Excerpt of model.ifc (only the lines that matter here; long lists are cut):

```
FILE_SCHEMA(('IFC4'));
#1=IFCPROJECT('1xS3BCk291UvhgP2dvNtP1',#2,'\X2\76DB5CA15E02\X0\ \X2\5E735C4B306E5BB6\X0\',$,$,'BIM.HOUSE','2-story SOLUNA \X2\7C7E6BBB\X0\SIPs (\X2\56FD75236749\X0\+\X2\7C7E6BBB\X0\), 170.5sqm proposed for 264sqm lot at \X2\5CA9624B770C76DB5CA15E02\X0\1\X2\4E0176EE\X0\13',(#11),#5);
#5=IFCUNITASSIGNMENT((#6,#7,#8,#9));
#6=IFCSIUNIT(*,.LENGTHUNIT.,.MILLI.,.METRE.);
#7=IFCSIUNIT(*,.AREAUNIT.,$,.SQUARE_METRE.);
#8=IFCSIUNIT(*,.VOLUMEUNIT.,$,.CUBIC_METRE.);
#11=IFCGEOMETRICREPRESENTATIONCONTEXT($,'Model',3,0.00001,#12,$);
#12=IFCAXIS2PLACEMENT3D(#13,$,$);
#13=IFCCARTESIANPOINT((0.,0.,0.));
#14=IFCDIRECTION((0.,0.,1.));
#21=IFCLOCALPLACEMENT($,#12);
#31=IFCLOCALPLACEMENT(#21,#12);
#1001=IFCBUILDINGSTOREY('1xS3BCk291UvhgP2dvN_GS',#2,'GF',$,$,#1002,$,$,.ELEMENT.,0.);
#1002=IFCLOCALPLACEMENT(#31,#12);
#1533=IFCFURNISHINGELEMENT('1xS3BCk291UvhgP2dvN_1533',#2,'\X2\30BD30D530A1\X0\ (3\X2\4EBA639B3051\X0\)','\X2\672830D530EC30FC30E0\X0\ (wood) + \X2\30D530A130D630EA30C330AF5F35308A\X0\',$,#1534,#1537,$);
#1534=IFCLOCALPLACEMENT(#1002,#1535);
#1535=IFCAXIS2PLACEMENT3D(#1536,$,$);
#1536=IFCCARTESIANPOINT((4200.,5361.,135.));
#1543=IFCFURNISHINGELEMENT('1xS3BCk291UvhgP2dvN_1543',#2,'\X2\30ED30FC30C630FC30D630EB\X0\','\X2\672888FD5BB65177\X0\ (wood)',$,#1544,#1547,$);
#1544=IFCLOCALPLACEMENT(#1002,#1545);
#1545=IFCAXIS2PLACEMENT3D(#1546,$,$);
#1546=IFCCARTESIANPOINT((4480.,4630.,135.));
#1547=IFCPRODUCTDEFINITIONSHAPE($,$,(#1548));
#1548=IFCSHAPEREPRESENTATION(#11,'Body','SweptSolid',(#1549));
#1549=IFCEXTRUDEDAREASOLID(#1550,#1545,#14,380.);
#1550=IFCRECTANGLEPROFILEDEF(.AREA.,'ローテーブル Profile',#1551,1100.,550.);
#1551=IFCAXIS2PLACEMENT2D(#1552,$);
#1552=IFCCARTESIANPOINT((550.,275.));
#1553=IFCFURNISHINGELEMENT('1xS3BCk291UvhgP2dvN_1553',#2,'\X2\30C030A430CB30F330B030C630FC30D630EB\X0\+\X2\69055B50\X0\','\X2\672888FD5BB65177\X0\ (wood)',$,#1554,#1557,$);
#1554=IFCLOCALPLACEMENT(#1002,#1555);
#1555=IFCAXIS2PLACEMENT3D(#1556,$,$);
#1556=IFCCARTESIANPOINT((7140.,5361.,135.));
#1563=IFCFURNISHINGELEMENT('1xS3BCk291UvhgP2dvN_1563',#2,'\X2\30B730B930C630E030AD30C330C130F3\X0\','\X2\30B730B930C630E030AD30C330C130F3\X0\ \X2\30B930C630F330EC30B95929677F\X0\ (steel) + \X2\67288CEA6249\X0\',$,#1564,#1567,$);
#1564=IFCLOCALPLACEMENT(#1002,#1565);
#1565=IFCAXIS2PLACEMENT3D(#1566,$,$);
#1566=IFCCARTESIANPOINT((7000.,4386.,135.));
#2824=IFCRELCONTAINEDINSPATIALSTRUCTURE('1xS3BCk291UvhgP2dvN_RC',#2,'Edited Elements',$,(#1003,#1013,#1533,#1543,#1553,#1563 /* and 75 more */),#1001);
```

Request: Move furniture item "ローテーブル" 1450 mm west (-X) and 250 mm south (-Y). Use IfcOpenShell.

```python
import ifcopenshell
import ifcopenshell.api.geometry
import ifcopenshell.util.placement

model = ifcopenshell.open("model.ifc")

item = model.by_guid("1xS3BCk291UvhgP2dvN_1543")
matrix = ifcopenshell.util.placement.get_local_placement(item.ObjectPlacement)
matrix[0, 3] -= 1450.0
matrix[1, 3] -= 250.0
ifcopenshell.api.geometry.edit_object_placement(model, product=item, matrix=matrix, is_si=False)

print(ifcopenshell.util.placement.get_local_placement(item.ObjectPlacement).round(3) + 0.0)

model.write("model_edited.ifc")
```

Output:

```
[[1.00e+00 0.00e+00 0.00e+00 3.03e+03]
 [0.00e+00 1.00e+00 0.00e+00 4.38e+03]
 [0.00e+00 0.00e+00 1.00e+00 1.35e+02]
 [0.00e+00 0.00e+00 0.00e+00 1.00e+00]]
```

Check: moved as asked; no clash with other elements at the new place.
